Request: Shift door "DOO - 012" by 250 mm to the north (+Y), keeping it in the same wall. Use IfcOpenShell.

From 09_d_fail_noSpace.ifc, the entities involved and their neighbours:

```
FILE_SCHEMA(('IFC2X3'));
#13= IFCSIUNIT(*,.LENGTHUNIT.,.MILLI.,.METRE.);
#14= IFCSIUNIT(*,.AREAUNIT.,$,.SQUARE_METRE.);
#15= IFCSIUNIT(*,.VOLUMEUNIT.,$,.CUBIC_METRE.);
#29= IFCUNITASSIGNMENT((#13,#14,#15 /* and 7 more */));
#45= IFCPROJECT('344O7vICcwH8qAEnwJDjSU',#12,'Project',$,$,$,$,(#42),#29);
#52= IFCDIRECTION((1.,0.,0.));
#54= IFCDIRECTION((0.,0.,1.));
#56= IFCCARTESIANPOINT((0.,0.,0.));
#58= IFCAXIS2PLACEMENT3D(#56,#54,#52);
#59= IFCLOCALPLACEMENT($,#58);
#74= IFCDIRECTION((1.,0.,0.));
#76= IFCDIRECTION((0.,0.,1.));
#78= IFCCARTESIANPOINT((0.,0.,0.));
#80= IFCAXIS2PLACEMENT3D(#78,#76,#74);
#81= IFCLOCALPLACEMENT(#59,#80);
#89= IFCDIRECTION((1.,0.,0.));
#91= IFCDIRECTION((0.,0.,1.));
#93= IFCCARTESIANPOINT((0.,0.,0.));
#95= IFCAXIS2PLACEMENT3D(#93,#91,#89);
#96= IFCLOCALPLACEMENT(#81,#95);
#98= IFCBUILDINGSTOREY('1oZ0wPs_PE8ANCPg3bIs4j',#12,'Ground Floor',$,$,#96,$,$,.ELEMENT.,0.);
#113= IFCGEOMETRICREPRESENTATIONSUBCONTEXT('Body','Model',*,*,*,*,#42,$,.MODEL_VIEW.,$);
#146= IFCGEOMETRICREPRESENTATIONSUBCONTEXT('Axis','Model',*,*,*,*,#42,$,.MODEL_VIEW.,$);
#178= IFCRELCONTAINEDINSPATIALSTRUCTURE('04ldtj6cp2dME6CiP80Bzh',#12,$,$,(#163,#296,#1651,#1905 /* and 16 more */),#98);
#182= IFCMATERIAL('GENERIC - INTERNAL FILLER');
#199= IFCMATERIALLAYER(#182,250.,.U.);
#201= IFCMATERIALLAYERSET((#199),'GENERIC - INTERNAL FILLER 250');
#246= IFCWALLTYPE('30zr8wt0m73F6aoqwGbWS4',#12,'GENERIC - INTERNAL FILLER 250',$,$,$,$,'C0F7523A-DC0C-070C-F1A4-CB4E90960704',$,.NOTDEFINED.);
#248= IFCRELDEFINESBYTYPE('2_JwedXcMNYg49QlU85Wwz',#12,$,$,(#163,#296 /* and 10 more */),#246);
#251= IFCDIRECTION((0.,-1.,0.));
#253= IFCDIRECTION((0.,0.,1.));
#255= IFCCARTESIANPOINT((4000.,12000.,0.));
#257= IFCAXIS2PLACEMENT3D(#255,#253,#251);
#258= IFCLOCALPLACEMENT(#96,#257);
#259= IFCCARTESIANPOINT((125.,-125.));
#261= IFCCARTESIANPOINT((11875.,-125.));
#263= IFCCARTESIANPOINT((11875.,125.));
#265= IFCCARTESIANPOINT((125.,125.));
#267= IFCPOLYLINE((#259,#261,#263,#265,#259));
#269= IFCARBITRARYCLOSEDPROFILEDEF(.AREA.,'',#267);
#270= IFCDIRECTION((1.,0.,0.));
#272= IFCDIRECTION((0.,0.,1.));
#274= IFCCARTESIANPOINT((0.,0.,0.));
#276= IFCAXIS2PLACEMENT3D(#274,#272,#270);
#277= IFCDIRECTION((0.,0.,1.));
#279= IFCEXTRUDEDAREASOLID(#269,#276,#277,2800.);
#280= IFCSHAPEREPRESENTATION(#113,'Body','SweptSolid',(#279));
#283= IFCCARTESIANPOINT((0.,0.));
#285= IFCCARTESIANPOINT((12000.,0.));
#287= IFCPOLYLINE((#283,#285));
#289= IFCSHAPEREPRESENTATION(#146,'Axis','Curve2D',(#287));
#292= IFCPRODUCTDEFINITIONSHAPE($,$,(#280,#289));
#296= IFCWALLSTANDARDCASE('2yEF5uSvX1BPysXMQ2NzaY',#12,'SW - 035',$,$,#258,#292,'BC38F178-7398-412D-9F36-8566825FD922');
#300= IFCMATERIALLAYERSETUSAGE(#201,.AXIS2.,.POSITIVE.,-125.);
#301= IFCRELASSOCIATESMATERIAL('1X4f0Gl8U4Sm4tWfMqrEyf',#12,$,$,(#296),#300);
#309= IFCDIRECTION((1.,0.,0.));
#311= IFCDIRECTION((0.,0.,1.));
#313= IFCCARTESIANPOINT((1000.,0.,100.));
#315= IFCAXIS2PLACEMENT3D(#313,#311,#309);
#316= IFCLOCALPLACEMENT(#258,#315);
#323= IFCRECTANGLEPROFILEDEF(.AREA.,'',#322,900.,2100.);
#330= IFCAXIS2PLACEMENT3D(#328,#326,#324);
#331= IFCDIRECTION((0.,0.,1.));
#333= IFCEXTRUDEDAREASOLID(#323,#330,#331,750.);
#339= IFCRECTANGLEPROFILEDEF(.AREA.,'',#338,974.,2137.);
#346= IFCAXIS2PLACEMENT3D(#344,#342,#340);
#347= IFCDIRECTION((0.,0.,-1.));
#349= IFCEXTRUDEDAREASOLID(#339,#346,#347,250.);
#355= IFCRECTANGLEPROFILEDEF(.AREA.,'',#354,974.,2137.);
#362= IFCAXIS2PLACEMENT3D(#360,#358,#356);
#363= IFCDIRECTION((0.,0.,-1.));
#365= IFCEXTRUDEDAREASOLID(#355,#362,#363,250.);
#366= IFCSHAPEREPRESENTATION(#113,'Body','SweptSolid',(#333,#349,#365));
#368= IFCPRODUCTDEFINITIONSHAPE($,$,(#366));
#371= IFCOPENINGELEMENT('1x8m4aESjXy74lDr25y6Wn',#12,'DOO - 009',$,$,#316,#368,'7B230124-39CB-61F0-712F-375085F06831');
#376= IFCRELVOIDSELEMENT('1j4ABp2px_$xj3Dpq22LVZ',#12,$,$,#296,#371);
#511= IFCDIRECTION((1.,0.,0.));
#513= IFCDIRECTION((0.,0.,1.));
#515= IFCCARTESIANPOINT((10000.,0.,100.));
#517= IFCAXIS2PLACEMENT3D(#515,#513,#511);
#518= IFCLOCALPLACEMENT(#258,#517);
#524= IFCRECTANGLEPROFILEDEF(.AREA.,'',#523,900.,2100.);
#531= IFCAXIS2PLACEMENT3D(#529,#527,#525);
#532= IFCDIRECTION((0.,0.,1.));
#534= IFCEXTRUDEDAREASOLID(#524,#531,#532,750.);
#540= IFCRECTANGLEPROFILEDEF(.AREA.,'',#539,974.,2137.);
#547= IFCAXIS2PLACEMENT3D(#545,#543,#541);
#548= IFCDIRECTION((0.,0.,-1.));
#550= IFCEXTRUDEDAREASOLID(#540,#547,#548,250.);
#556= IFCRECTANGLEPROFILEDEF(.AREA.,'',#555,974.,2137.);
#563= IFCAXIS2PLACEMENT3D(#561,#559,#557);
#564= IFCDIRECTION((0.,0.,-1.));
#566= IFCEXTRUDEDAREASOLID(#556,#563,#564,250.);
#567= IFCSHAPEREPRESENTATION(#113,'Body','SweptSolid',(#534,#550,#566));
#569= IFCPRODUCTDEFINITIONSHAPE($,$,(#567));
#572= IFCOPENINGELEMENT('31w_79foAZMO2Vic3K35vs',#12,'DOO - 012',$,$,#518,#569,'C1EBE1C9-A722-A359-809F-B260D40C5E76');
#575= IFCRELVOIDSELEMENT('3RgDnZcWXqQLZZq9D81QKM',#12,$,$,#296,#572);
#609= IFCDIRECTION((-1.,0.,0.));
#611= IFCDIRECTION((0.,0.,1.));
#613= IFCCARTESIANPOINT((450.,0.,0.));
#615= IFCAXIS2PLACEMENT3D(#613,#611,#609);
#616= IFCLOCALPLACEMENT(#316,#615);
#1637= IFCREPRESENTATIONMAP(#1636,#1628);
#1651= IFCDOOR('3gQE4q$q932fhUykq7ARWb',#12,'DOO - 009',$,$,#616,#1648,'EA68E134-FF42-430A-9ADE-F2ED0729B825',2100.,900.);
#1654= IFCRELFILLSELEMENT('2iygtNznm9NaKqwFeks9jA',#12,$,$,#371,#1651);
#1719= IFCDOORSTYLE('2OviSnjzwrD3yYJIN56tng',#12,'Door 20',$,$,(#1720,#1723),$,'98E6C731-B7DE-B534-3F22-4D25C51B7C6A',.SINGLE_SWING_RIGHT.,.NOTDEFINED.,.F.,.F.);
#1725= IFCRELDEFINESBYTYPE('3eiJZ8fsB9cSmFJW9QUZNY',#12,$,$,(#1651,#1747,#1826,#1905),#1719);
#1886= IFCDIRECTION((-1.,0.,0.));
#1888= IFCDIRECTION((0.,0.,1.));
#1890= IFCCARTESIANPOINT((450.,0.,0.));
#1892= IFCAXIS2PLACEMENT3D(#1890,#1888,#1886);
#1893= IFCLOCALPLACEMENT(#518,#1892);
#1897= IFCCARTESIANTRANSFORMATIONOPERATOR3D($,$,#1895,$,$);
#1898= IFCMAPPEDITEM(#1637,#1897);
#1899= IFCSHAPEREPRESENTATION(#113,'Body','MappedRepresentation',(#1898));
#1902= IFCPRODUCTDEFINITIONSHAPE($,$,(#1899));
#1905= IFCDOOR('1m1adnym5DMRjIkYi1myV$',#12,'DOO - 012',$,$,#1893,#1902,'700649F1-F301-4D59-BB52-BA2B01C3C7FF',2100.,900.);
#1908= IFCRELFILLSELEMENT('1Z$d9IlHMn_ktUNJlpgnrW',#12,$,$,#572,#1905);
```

```python
import ifcopenshell
import ifcopenshell.api.geometry
import ifcopenshell.util.placement
import ifcopenshell.util.unit

model = ifcopenshell.open("09_d_fail_noSpace.ifc")
unit_scale = ifcopenshell.util.unit.calculate_unit_scale(model)

door = model.by_guid("1m1adnym5DMRjIkYi1myV$")
opening = door.FillsVoids[0].RelatingOpeningElement
wall = opening.VoidsElements[0].RelatingBuildingElement

wall_matrix = ifcopenshell.util.placement.get_local_placement(wall.ObjectPlacement)
shift = wall_matrix[:3, 0] * -0.25 / unit_scale
before = ifcopenshell.util.placement.get_local_placement(door.ObjectPlacement)[:3, 3].copy()

# The door is placed relative to its opening, so it follows when the opening moves.
matrix = ifcopenshell.util.placement.get_local_placement(opening.ObjectPlacement)
matrix[:3, 3] += shift
ifcopenshell.api.geometry.edit_object_placement(
    model, product=opening, matrix=matrix, is_si=False, should_transform_children=True
)

after = ifcopenshell.util.placement.get_local_placement(door.ObjectPlacement)[:3, 3]
print("door moved by", (after - before).round(3) + 0.0)

model.write("09_d_fail_noSpace_edited.ifc")
```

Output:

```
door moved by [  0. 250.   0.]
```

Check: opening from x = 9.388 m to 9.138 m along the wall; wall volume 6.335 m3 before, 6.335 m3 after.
